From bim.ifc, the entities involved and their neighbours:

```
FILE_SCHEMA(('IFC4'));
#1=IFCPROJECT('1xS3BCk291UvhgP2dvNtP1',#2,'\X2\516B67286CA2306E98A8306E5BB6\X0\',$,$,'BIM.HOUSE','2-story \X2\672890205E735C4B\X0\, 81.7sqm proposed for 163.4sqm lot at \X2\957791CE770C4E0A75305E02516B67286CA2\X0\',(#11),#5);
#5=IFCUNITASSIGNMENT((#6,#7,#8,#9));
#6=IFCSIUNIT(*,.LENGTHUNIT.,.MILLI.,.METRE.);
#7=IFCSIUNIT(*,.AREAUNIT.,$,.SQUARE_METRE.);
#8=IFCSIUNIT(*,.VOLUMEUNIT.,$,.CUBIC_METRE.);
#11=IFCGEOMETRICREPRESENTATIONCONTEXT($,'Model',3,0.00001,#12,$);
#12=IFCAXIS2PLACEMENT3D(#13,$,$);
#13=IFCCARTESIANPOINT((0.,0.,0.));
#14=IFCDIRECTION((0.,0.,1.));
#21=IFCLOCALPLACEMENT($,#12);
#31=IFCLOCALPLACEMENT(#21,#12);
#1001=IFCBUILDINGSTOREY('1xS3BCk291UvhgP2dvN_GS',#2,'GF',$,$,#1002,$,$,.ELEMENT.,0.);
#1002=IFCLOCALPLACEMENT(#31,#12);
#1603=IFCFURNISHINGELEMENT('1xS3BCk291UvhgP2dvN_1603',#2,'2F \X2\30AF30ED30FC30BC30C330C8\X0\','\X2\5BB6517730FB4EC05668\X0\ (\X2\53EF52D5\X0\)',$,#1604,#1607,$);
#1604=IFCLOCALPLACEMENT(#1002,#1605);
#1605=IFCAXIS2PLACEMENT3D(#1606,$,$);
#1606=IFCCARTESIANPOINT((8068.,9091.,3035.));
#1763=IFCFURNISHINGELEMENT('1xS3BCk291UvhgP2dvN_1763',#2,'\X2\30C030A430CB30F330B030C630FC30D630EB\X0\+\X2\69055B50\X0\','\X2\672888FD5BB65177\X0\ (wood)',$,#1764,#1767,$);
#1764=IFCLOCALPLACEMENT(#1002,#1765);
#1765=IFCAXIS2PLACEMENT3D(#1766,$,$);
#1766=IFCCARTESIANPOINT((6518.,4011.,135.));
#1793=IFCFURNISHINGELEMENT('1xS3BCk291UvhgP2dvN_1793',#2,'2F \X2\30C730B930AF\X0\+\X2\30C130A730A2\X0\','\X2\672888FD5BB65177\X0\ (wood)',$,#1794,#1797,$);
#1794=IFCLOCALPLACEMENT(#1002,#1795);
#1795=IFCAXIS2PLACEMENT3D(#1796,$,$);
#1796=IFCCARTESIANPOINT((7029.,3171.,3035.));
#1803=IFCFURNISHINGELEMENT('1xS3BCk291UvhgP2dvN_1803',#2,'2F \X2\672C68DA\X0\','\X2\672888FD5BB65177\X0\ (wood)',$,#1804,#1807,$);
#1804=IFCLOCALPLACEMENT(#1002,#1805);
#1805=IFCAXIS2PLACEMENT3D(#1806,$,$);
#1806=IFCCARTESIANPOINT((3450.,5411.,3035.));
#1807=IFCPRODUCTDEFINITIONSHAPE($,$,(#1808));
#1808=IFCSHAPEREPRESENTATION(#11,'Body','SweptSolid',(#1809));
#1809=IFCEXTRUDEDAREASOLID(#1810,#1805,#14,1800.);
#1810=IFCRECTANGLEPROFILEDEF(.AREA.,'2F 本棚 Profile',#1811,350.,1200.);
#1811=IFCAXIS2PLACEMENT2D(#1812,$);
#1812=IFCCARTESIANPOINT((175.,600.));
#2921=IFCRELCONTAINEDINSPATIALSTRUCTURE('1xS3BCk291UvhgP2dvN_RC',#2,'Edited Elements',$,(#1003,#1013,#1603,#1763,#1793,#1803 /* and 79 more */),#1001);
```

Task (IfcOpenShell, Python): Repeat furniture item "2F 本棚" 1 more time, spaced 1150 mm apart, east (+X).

```python
import numpy as np
import ifcopenshell
import ifcopenshell.api.geometry
import ifcopenshell.api.root
import ifcopenshell.util.element
import ifcopenshell.util.placement
import ifcopenshell.util.unit

model = ifcopenshell.open("bim.ifc")
unit_scale = ifcopenshell.util.unit.calculate_unit_scale(model)


def reuse_history(source, copy):
    """copy_class also copies each property set's owner history, people and application; keep the originals."""
    for rel in copy.IsDefinedBy:
        if rel.is_a("IfcRelDefinesByProperties") and (history := rel.RelatingPropertyDefinition.OwnerHistory):
            rel.RelatingPropertyDefinition.OwnerHistory = source.OwnerHistory
            ifcopenshell.util.element.remove_deep2(model, history)


source = model.by_id(1803)
base = ifcopenshell.util.placement.get_local_placement(source.ObjectPlacement)
step = np.array([1.0, 0.0, 0.0]) * 1.15 / unit_scale

for i in range(1, 2):
    copy = ifcopenshell.api.root.copy_class(model, product=source)
    copy.Representation = ifcopenshell.util.element.copy_deep(
        model, source.Representation, exclude=["IfcGeometricRepresentationContext", "IfcRepresentationMap"]
    )
    reuse_history(source, copy)
    matrix = base.copy()
    matrix[:3, 3] += i * step
    print("added at", matrix[:3, 3].round(3) + 0.0)
    ifcopenshell.api.geometry.edit_object_placement(model, product=copy, matrix=matrix, is_si=False)

model.write("bim_rev.ifc")
```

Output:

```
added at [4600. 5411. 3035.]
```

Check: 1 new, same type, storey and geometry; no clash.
